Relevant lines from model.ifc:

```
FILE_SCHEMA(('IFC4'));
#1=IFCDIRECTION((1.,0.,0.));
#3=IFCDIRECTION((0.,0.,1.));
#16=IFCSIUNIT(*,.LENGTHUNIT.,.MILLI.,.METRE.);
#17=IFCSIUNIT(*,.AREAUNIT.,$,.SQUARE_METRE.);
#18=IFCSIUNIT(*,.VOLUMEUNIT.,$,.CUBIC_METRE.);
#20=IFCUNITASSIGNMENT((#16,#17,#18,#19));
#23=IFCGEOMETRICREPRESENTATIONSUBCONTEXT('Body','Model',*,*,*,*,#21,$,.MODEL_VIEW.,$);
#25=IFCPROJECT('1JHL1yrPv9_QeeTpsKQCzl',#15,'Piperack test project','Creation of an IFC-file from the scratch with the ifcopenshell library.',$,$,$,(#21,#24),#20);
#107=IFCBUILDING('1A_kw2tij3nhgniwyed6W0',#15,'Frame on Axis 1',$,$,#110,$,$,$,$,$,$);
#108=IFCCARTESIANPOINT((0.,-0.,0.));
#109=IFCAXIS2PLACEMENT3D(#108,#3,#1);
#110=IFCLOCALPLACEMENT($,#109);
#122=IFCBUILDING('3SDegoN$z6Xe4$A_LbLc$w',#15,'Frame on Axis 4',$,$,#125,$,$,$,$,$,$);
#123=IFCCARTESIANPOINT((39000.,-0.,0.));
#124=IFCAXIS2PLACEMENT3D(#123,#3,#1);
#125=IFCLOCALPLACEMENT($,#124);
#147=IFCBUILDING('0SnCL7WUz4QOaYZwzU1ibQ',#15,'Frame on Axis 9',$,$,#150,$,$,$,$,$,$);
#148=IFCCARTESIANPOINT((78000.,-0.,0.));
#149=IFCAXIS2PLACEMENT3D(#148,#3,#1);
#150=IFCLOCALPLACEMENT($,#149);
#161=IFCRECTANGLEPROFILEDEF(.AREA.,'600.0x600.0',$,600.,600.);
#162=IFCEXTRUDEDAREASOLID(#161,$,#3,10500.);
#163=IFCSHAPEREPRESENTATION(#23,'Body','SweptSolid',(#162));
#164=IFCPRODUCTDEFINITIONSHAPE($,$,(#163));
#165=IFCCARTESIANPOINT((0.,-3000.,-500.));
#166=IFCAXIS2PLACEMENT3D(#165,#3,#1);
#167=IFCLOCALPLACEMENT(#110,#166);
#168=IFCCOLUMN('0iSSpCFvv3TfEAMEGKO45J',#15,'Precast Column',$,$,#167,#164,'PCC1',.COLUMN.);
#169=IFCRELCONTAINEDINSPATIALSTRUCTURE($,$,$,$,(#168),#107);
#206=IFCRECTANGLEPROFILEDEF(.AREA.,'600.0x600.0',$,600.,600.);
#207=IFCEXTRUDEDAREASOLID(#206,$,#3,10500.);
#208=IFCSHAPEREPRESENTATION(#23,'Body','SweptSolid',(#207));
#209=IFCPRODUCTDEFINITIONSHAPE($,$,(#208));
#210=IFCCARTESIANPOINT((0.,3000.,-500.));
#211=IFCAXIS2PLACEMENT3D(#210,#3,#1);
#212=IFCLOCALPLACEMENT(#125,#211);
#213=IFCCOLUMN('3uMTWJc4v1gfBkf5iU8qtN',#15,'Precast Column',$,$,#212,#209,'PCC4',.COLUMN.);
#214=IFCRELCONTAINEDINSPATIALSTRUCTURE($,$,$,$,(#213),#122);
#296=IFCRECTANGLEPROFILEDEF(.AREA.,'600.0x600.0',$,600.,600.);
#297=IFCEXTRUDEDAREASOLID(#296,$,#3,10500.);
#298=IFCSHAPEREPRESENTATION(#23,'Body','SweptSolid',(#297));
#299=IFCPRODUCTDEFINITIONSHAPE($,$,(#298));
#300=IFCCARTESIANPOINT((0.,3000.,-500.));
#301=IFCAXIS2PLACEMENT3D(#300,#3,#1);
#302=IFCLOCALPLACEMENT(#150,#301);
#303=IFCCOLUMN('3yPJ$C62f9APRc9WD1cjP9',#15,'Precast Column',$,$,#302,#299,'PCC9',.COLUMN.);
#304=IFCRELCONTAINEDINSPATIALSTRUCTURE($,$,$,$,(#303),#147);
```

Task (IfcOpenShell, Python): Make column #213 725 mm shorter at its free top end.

```python
import ifcopenshell
import ifcopenshell.util.representation
import ifcopenshell.util.unit

model = ifcopenshell.open("model.ifc")
unit_scale = ifcopenshell.util.unit.calculate_unit_scale(model)

member = model.by_guid("3uMTWJc4v1gfBkf5iU8qtN")
change = -0.725 / unit_scale

# The extrusion runs towards the end named, so only its depth changes.
body = ifcopenshell.util.representation.get_representation(member, "Model", "Body")
solid = body.Items[0]
old_length = solid.Depth
solid.Depth += change

print(f"length {old_length:g} -> {solid.Depth:g}")

model.write("model_updated.ifc")
```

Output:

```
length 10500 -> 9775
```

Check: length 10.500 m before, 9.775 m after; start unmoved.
